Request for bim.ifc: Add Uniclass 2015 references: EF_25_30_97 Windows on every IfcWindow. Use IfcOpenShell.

First a look at what the model holds.

```python
import ifcopenshell

model = ifcopenshell.open("bim.ifc")
print(model.schema)
print("classifications:", [c.Name for c in model.by_type("IfcClassification")])
for ifc_class in ("IfcDoor", "IfcRoof", "IfcStair", "IfcWall", "IfcWindow"):
    print(ifc_class, len(model.by_type(ifc_class)))
```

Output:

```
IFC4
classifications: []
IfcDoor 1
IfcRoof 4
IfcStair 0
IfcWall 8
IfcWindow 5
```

```python
import ifcopenshell
import ifcopenshell.api.classification

model = ifcopenshell.open("bim.ifc")

system = ifcopenshell.api.classification.add_classification(model, classification="Uniclass 2015")

codes = {
    "IfcWindow": ("EF_25_30_97", "Windows"),
}
for ifc_class, (code, name) in codes.items():
    products = model.by_type(ifc_class)
    ifcopenshell.api.classification.add_reference(
        model, products=products, classification=system, identification=code, name=name
    )
    print(code, len(products))

model.write("bim_rev.ifc")
```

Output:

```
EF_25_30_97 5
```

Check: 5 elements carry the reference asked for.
